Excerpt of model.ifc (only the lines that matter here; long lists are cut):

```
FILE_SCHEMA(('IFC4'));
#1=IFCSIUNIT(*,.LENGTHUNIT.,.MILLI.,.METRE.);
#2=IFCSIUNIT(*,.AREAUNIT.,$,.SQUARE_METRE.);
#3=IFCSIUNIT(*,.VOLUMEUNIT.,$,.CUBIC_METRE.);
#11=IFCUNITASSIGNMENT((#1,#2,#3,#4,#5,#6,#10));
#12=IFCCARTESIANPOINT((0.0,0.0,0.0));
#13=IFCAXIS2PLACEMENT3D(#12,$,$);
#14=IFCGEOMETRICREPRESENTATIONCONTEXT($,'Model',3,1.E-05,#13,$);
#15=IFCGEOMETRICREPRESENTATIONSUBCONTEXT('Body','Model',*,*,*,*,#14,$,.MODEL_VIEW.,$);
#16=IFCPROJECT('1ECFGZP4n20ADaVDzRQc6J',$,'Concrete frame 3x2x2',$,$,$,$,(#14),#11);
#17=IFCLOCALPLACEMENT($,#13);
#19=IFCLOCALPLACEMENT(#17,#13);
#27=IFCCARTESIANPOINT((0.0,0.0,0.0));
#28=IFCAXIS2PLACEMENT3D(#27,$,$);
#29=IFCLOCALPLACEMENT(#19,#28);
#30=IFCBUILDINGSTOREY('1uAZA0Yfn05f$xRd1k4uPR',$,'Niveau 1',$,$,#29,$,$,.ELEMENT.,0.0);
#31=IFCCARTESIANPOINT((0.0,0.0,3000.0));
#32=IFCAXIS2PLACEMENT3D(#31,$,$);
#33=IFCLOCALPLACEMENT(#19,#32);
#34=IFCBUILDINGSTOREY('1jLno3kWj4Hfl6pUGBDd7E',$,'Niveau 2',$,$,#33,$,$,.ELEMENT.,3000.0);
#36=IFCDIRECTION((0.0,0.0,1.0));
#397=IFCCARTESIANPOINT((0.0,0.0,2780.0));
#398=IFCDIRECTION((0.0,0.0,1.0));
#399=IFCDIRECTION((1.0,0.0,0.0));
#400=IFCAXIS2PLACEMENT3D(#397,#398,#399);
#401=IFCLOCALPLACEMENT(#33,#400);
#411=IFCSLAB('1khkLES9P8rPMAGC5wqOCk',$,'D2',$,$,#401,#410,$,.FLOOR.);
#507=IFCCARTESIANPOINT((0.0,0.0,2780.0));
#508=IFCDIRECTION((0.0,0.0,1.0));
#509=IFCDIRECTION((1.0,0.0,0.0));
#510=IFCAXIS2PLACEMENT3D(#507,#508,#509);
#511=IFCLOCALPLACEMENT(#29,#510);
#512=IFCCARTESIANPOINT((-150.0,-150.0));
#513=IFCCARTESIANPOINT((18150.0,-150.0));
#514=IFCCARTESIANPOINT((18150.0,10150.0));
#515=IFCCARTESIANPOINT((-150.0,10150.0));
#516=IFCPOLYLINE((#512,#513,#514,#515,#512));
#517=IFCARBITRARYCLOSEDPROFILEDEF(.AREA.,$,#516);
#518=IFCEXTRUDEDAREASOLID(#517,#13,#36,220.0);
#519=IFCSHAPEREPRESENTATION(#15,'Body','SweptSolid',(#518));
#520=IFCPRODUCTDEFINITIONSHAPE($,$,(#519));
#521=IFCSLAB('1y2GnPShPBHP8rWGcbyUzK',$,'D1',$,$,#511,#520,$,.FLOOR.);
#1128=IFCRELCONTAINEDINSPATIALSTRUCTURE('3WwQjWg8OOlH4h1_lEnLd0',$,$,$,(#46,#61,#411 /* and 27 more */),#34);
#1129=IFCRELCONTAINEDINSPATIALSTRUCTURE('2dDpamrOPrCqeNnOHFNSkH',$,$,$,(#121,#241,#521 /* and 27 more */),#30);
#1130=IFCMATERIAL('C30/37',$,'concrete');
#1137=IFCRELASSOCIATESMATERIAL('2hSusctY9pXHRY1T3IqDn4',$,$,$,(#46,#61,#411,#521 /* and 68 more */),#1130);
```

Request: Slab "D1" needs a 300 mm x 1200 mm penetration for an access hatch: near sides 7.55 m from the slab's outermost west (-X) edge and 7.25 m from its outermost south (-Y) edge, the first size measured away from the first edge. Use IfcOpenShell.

```python
import numpy as np
import ifcopenshell
import ifcopenshell.api.feature
import ifcopenshell.api.geometry
import ifcopenshell.api.root
import ifcopenshell.geom
import ifcopenshell.util.placement
import ifcopenshell.util.representation
import ifcopenshell.util.shape
import ifcopenshell.util.unit

model = ifcopenshell.open("model.ifc")
unit_scale = ifcopenshell.util.unit.calculate_unit_scale(model)
settings = ifcopenshell.geom.settings()


def volume(element):
    """Net volume in cubic metres, openings subtracted."""
    shape = ifcopenshell.geom.create_shape(settings, element)
    return ifcopenshell.util.shape.get_volume(shape.geometry)


slab = model.by_guid("1y2GnPShPBHP8rWGcbyUzK")
before = volume(slab)

# Extent in the slab's own axes, in metres. The edges named are its -X and -Y sides.
slab_shape = ifcopenshell.geom.create_shape(settings, slab)
vertices = ifcopenshell.util.shape.get_vertices(slab_shape.geometry)
x_min, y_min, bottom = vertices.min(axis=0)
top = vertices[:, 2].max()

opening = ifcopenshell.api.root.create_entity(model, ifc_class="IfcOpeningElement", name="Access hatch opening", predefined_type="OPENING")
context = ifcopenshell.util.representation.get_context(model, "Model", "Body", "MODEL_VIEW")
width, depth = 0.3, 1.2
outline = [(0.0, 0.0), (width, 0.0), (width, depth), (0.0, depth), (0.0, 0.0)]
# Overshoot both faces by 50 mm so the cut is clean.
shape = ifcopenshell.api.geometry.add_slab_representation(
    model, context=context, depth=top - bottom + 0.1, polyline=outline
)
ifcopenshell.api.geometry.assign_representation(model, product=opening, representation=shape)

matrix = ifcopenshell.util.placement.get_local_placement(slab.ObjectPlacement)
matrix[:, 3] = matrix @ np.append(np.array([x_min + 7.55, y_min + 7.25, bottom - 0.05]) / unit_scale, 1.0)
ifcopenshell.api.geometry.edit_object_placement(model, product=opening, matrix=matrix, is_si=False)
ifcopenshell.api.feature.add_feature(model, feature=opening, element=slab)

after = volume(slab)

print(f"slab volume {before:.3f} -> {after:.3f} m3")

model.write("model_updated.ifc")
```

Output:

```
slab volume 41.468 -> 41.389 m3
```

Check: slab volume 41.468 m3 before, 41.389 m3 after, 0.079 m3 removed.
